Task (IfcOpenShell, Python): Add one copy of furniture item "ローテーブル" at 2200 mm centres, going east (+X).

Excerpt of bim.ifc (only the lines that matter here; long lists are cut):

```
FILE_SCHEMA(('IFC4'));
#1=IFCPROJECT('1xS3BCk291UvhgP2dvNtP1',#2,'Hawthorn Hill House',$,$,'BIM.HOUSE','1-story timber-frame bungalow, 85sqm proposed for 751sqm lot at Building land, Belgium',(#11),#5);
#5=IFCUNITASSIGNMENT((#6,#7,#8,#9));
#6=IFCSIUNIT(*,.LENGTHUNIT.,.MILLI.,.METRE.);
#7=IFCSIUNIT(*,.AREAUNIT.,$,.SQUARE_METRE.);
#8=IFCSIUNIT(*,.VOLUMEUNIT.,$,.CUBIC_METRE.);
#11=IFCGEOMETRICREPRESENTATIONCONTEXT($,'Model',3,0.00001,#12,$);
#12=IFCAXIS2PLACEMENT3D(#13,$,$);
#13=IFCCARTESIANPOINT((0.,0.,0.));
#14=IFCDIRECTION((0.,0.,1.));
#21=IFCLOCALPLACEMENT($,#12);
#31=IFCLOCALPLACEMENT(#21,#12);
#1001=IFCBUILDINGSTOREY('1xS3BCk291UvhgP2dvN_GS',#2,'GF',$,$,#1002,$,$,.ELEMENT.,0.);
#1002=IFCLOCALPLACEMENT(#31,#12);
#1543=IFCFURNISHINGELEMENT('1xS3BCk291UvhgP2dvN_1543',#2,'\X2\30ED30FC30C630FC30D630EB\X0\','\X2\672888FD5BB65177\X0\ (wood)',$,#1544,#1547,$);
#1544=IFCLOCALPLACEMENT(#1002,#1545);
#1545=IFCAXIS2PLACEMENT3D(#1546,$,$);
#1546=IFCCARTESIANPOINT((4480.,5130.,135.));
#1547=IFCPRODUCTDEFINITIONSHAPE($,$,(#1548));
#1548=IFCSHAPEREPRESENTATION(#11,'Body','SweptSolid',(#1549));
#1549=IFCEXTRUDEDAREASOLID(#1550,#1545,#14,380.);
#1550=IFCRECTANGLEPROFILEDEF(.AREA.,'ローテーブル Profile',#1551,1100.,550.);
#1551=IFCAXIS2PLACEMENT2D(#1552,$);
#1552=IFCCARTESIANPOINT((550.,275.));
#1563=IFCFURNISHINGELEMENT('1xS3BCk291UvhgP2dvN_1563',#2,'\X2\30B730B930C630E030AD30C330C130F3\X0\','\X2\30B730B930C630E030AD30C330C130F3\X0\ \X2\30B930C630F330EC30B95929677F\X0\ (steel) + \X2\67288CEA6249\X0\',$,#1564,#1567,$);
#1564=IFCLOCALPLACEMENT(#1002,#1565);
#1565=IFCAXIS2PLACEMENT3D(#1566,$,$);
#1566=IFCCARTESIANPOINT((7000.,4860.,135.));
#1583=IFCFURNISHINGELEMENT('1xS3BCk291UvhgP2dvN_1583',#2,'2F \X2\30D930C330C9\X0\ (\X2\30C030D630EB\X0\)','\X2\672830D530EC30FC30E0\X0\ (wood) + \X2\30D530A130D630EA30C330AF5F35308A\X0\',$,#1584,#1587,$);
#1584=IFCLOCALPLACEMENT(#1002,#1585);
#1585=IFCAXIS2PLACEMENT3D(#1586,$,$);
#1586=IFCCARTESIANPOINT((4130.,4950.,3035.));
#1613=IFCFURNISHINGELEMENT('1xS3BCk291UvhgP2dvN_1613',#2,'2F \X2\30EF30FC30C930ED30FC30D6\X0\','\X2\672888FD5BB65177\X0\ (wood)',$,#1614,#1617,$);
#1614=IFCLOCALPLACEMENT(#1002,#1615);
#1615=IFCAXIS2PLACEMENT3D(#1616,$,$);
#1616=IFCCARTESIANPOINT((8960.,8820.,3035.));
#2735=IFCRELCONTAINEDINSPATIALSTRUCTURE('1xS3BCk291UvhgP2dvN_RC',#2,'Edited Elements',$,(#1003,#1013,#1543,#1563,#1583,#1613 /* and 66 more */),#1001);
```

```python
import numpy as np
import ifcopenshell
import ifcopenshell.api.geometry
import ifcopenshell.api.root
import ifcopenshell.util.element
import ifcopenshell.util.placement
import ifcopenshell.util.unit

model = ifcopenshell.open("bim.ifc")
unit_scale = ifcopenshell.util.unit.calculate_unit_scale(model)


def reuse_history(source, copy):
    """copy_class also copies each property set's owner history, people and application; keep the originals."""
    for rel in copy.IsDefinedBy:
        if rel.is_a("IfcRelDefinesByProperties") and (history := rel.RelatingPropertyDefinition.OwnerHistory):
            rel.RelatingPropertyDefinition.OwnerHistory = source.OwnerHistory
            ifcopenshell.util.element.remove_deep2(model, history)


source = model.by_id(1543)
base = ifcopenshell.util.placement.get_local_placement(source.ObjectPlacement)
step = np.array([1.0, 0.0, 0.0]) * 2.2 / unit_scale

for i in range(1, 2):
    copy = ifcopenshell.api.root.copy_class(model, product=source)
    copy.Representation = ifcopenshell.util.element.copy_deep(
        model, source.Representation, exclude=["IfcGeometricRepresentationContext", "IfcRepresentationMap"]
    )
    reuse_history(source, copy)
    matrix = base.copy()
    matrix[:3, 3] += i * step
    print("added at", matrix[:3, 3].round(3) + 0.0)
    ifcopenshell.api.geometry.edit_object_placement(model, product=copy, matrix=matrix, is_si=False)

model.write("bim_updated.ifc")
```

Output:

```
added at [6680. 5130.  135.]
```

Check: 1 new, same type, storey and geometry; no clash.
